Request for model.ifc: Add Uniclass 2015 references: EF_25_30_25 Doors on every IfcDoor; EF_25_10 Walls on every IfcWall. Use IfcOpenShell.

First a look at what the model holds.

```python
import ifcopenshell

model = ifcopenshell.open("model.ifc")
print(model.schema)
print("classifications:", [c.Name for c in model.by_type("IfcClassification")])
for ifc_class in ("IfcDoor", "IfcRoof", "IfcStair", "IfcWall", "IfcWindow"):
    print(ifc_class, len(model.by_type(ifc_class)))
```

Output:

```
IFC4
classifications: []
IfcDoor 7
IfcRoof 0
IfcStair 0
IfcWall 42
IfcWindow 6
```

```python
import ifcopenshell
import ifcopenshell.api.classification

model = ifcopenshell.open("model.ifc")

system = ifcopenshell.api.classification.add_classification(model, classification="Uniclass 2015")

codes = {
    "IfcDoor": ("EF_25_30_25", "Doors"),
    "IfcWall": ("EF_25_10", "Walls"),
}
for ifc_class, (code, name) in codes.items():
    products = model.by_type(ifc_class)
    ifcopenshell.api.classification.add_reference(
        model, products=products, classification=system, identification=code, name=name
    )
    print(code, len(products))

model.write("model_updated.ifc")
```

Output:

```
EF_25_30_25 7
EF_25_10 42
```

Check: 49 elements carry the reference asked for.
